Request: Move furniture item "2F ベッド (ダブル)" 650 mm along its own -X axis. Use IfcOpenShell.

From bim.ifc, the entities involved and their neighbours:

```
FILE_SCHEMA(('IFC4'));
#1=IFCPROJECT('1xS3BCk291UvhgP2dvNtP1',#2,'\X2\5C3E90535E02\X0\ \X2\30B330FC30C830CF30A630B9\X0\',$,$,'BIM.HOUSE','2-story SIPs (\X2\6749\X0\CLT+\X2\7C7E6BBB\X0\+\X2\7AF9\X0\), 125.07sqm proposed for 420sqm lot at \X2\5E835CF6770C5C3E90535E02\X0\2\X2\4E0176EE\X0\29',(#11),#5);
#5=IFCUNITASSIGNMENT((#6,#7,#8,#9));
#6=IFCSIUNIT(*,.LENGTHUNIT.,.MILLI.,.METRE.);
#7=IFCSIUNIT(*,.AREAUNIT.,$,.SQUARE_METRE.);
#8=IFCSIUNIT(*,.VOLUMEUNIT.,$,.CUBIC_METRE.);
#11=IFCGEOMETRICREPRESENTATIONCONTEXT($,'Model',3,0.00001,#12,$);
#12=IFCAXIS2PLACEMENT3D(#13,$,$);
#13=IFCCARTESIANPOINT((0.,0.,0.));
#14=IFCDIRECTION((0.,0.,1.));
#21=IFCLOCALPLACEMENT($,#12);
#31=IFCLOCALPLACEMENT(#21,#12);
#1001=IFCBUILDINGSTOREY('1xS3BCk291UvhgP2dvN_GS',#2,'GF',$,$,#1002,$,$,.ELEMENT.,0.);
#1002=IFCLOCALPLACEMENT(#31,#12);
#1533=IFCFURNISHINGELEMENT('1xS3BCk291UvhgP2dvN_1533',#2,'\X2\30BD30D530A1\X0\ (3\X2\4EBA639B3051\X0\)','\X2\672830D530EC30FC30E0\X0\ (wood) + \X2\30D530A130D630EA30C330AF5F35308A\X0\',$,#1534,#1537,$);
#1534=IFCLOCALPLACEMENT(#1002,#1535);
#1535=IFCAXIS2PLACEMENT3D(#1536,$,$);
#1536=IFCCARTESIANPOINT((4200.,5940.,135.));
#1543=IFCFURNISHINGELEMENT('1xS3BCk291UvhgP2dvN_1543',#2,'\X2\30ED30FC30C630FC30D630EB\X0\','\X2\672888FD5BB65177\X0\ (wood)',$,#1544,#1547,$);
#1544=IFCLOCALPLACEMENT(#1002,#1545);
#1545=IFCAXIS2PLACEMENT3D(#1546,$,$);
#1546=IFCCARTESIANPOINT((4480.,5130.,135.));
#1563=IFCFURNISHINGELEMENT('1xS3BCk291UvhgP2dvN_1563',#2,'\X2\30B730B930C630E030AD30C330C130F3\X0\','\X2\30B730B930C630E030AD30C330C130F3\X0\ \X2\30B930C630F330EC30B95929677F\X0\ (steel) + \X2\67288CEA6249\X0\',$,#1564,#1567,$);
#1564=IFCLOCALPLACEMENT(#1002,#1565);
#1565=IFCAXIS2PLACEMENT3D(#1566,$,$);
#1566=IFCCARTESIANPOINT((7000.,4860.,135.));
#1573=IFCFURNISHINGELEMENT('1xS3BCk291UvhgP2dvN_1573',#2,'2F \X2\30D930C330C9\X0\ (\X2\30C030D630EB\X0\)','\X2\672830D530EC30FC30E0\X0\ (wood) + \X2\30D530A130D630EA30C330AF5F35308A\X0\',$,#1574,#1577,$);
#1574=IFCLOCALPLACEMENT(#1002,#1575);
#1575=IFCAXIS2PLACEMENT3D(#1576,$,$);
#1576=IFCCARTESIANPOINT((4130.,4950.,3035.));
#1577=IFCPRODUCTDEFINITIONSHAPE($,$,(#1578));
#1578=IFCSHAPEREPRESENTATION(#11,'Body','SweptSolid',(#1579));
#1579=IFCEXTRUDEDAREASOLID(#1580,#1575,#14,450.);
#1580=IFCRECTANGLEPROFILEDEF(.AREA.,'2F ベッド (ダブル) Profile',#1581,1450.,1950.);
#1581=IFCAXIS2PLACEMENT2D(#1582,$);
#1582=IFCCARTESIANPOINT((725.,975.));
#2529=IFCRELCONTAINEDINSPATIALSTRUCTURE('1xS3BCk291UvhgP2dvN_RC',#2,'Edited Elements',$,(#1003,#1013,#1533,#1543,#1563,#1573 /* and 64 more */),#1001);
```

```python
import ifcopenshell
import ifcopenshell.api.geometry
import ifcopenshell.util.placement

model = ifcopenshell.open("bim.ifc")

item = model.by_id(1573)
matrix = ifcopenshell.util.placement.get_local_placement(item.ObjectPlacement)
matrix[:3, 3] -= matrix[:3, 0] * 650.0
ifcopenshell.api.geometry.edit_object_placement(model, product=item, matrix=matrix, is_si=False)

print(ifcopenshell.util.placement.get_local_placement(item.ObjectPlacement).round(3) + 0.0)

model.write("bim_v2.ifc")
```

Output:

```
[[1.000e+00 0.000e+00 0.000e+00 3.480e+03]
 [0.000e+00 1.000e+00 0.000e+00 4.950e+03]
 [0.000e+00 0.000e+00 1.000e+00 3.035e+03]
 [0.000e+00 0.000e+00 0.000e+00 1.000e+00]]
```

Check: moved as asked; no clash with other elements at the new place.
